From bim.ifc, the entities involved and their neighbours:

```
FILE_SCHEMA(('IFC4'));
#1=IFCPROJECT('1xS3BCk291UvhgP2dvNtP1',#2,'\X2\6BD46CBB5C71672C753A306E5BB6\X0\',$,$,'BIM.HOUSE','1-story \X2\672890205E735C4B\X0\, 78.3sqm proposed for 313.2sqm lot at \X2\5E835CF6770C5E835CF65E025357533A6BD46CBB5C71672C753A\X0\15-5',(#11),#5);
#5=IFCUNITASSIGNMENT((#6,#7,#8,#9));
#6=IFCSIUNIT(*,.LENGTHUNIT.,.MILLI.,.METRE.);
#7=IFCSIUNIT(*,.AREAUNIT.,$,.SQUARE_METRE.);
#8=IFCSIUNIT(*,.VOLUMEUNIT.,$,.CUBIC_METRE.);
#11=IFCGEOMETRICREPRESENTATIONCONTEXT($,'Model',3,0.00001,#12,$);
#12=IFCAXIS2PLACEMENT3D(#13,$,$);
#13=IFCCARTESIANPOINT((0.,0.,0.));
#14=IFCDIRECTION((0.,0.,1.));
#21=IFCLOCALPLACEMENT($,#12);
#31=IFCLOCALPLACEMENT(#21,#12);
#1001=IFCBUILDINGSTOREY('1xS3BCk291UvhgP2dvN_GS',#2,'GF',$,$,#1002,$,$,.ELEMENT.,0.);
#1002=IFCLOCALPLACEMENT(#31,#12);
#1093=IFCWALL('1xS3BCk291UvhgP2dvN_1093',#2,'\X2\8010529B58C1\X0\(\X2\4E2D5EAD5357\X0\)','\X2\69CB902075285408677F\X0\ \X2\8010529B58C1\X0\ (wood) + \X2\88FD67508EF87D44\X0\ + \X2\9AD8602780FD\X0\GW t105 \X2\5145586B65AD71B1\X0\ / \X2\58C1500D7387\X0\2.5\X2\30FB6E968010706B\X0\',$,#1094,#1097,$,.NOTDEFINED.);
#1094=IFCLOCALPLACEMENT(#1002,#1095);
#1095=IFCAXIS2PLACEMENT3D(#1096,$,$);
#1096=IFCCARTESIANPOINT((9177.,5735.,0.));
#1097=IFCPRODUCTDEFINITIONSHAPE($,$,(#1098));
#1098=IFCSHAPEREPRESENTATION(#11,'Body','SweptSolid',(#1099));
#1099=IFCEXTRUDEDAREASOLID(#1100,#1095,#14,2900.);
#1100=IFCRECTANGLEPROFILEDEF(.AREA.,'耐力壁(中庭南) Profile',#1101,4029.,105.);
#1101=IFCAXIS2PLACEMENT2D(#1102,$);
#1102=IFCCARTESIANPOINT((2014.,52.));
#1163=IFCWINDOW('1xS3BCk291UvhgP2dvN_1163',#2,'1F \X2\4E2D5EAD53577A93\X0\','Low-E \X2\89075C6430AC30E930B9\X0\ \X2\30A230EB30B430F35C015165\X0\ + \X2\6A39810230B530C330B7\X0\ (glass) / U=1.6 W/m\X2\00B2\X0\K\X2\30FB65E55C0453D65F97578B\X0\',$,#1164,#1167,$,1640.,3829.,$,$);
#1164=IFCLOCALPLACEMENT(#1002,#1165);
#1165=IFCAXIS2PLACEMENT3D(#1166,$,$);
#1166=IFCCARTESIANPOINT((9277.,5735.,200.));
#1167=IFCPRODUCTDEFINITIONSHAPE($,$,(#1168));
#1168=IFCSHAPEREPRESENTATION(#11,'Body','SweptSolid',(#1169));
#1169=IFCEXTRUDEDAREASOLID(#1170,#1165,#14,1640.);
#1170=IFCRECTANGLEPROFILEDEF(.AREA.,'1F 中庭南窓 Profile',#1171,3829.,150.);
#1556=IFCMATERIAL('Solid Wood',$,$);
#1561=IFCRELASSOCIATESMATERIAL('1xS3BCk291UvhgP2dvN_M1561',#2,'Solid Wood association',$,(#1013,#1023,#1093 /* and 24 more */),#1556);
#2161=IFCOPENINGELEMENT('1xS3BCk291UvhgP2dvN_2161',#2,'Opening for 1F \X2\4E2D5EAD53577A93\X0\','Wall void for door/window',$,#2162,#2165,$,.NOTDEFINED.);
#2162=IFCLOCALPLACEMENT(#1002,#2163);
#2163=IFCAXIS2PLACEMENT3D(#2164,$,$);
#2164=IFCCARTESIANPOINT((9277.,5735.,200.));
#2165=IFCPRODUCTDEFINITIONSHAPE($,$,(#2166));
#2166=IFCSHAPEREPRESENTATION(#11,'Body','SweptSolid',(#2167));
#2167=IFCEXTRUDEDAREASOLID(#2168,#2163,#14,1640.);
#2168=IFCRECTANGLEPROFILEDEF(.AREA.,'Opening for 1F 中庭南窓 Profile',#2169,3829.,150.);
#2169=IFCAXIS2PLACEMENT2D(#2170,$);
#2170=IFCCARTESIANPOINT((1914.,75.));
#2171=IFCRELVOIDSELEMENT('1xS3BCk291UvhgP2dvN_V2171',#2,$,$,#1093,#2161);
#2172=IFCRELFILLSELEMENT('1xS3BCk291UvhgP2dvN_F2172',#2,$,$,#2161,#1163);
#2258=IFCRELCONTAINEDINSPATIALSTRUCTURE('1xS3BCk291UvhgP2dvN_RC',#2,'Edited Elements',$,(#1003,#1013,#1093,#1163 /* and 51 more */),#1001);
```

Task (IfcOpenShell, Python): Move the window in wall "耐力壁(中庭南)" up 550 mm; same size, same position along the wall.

```python
import numpy as np
import ifcopenshell
import ifcopenshell.api.geometry
import ifcopenshell.util.placement
import ifcopenshell.util.unit

model = ifcopenshell.open("bim.ifc")
unit_scale = ifcopenshell.util.unit.calculate_unit_scale(model)

window = model.by_id(1163)
opening = window.FillsVoids[0].RelatingOpeningElement
dz = 550.0

shift = np.array([0.0, 0.0, dz])
# The window is not placed relative to its opening, so move both.
for product in (opening, window):
    matrix = ifcopenshell.util.placement.get_local_placement(product.ObjectPlacement)
    matrix[:3, 3] += shift
    ifcopenshell.api.geometry.edit_object_placement(model, product=product, matrix=matrix, is_si=False)

print(f"moved by {dz * unit_scale:+.3f} m")

model.write("bim-out.ifc")
```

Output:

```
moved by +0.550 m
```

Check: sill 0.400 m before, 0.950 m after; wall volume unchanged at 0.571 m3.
